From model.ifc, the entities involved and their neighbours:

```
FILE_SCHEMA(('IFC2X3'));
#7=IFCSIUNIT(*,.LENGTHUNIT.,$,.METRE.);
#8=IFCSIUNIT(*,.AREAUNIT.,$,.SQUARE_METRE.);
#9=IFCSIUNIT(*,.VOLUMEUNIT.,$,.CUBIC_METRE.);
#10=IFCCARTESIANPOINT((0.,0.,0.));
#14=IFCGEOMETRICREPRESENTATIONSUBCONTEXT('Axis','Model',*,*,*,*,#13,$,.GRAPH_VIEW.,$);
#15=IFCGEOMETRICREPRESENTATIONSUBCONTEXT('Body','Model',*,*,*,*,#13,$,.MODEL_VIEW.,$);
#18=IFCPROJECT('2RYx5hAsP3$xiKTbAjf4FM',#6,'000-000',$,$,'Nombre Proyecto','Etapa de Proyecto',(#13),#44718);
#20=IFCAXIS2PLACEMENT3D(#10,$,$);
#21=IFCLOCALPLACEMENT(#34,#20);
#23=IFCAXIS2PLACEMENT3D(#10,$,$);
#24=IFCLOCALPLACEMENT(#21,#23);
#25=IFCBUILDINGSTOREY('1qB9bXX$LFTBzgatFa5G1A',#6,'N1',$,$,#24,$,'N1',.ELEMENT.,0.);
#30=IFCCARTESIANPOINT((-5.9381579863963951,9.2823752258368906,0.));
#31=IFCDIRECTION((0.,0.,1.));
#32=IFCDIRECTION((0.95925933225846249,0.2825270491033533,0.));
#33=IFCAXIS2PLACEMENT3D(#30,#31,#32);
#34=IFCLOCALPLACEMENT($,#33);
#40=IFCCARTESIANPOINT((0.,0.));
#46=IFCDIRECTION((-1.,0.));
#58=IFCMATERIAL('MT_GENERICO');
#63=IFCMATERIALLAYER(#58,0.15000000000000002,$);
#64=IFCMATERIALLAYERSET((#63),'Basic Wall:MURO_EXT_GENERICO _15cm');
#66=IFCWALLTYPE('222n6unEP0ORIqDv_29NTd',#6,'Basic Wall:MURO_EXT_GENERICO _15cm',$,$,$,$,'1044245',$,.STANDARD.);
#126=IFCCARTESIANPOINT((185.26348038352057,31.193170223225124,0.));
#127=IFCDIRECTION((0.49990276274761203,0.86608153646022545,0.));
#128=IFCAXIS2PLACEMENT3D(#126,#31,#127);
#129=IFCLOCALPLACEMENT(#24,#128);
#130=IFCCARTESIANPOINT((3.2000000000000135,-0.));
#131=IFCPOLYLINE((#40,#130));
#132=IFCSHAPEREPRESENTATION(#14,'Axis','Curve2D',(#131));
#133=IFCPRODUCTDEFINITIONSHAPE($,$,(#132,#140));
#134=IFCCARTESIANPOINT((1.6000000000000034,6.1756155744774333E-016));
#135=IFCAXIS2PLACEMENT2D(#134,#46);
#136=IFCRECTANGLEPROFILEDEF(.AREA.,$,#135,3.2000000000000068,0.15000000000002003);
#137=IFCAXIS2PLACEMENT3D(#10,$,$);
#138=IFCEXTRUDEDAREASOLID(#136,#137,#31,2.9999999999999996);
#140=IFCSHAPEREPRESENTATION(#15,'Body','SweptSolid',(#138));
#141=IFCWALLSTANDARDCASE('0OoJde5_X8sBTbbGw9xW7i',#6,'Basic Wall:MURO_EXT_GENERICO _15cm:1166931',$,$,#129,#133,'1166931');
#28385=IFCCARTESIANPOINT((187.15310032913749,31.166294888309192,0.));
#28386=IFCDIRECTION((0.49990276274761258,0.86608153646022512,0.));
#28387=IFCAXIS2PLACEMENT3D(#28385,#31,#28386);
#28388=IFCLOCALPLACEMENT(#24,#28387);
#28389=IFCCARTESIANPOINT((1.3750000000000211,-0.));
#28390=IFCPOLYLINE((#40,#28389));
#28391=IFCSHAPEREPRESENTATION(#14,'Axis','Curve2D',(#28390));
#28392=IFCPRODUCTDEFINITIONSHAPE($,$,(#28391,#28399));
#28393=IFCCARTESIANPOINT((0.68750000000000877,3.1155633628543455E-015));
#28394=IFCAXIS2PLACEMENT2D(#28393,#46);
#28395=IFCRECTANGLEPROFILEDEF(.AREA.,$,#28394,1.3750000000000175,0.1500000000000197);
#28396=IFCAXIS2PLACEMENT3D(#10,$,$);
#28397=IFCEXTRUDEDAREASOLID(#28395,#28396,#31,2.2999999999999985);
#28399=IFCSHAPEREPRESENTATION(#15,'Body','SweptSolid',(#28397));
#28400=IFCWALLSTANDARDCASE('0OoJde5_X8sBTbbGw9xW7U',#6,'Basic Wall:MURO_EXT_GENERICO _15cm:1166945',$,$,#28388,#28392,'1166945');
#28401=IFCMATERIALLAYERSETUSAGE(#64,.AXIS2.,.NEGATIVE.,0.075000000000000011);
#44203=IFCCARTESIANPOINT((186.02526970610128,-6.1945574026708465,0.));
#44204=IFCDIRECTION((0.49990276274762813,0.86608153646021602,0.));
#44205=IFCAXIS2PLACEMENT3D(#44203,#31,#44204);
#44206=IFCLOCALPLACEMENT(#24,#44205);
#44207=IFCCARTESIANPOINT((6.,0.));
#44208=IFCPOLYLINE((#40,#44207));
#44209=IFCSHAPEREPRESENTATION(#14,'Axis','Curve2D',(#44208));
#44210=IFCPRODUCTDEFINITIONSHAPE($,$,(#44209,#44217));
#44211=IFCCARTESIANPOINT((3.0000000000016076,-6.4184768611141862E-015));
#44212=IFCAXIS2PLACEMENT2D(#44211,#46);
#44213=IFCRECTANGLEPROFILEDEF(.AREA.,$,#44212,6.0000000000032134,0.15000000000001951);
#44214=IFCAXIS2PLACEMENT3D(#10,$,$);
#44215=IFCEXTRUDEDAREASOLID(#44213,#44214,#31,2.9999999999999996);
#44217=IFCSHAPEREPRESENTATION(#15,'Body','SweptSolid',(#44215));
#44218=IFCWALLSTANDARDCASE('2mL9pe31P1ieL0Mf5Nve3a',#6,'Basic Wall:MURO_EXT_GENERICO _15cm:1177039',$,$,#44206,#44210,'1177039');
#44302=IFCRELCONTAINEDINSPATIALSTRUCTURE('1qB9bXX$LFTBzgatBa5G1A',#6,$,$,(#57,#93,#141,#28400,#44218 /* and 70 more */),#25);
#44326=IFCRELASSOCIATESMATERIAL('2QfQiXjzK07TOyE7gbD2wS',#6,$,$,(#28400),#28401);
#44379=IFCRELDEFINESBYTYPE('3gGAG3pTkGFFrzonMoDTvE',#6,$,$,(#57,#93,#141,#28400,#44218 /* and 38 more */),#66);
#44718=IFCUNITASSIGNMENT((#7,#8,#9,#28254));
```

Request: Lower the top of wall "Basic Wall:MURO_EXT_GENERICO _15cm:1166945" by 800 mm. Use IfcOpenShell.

```python
import ifcopenshell
import ifcopenshell.geom
import ifcopenshell.util.representation
import ifcopenshell.util.shape
import ifcopenshell.util.unit

model = ifcopenshell.open("model.ifc")
unit_scale = ifcopenshell.util.unit.calculate_unit_scale(model)
settings = ifcopenshell.geom.settings()


def volume(element):
    """Net volume in cubic metres, openings subtracted."""
    shape = ifcopenshell.geom.create_shape(settings, element)
    return ifcopenshell.util.shape.get_volume(shape.geometry)


wall = model.by_id(28400)
before = volume(wall)

body = ifcopenshell.util.representation.get_representation(wall, "Model", "Body")
solid = body.Items[0]
old_height = solid.Depth
solid.Depth -= 0.8 / unit_scale
after = volume(wall)

print(f"height {old_height:g} -> {solid.Depth:g}, volume {before:.3f} -> {after:.3f} m3")

model.write("model_updated.ifc")
```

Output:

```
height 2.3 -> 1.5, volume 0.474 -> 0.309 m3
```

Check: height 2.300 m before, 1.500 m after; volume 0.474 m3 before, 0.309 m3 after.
